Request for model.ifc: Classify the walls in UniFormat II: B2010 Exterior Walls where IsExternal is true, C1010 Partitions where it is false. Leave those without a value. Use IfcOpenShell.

First a look at what the model holds.

```python
import ifcopenshell
import ifcopenshell.util.element

model = ifcopenshell.open("model.ifc")
print(model.schema)
print("classifications:", [c.Name for c in model.by_type("IfcClassification")])
values = [ifcopenshell.util.element.get_pset(e, "Pset_WallCommon", "IsExternal") for e in model.by_type("IfcWall")]
for value in (True, False, None):
    print("IsExternal", value, values.count(value))
```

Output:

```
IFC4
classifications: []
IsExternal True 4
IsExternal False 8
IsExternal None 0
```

```python
import ifcopenshell
import ifcopenshell.api.classification
import ifcopenshell.util.element

model = ifcopenshell.open("model.ifc")

system = ifcopenshell.api.classification.add_classification(model, classification="UniFormat II")

walls = model.by_type("IfcWall")
external = {e: ifcopenshell.util.element.get_pset(e, "Pset_WallCommon", "IsExternal") for e in walls}
for flag, code, name in ((True, "B2010", "Exterior Walls"), (False, "C1010", "Partitions")):
    products = [e for e in walls if external[e] is flag]
    ifcopenshell.api.classification.add_reference(
        model, products=products, classification=system, identification=code, name=name
    )
    print(code, len(products))

model.write("model_updated.ifc")
```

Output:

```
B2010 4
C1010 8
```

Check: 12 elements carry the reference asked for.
